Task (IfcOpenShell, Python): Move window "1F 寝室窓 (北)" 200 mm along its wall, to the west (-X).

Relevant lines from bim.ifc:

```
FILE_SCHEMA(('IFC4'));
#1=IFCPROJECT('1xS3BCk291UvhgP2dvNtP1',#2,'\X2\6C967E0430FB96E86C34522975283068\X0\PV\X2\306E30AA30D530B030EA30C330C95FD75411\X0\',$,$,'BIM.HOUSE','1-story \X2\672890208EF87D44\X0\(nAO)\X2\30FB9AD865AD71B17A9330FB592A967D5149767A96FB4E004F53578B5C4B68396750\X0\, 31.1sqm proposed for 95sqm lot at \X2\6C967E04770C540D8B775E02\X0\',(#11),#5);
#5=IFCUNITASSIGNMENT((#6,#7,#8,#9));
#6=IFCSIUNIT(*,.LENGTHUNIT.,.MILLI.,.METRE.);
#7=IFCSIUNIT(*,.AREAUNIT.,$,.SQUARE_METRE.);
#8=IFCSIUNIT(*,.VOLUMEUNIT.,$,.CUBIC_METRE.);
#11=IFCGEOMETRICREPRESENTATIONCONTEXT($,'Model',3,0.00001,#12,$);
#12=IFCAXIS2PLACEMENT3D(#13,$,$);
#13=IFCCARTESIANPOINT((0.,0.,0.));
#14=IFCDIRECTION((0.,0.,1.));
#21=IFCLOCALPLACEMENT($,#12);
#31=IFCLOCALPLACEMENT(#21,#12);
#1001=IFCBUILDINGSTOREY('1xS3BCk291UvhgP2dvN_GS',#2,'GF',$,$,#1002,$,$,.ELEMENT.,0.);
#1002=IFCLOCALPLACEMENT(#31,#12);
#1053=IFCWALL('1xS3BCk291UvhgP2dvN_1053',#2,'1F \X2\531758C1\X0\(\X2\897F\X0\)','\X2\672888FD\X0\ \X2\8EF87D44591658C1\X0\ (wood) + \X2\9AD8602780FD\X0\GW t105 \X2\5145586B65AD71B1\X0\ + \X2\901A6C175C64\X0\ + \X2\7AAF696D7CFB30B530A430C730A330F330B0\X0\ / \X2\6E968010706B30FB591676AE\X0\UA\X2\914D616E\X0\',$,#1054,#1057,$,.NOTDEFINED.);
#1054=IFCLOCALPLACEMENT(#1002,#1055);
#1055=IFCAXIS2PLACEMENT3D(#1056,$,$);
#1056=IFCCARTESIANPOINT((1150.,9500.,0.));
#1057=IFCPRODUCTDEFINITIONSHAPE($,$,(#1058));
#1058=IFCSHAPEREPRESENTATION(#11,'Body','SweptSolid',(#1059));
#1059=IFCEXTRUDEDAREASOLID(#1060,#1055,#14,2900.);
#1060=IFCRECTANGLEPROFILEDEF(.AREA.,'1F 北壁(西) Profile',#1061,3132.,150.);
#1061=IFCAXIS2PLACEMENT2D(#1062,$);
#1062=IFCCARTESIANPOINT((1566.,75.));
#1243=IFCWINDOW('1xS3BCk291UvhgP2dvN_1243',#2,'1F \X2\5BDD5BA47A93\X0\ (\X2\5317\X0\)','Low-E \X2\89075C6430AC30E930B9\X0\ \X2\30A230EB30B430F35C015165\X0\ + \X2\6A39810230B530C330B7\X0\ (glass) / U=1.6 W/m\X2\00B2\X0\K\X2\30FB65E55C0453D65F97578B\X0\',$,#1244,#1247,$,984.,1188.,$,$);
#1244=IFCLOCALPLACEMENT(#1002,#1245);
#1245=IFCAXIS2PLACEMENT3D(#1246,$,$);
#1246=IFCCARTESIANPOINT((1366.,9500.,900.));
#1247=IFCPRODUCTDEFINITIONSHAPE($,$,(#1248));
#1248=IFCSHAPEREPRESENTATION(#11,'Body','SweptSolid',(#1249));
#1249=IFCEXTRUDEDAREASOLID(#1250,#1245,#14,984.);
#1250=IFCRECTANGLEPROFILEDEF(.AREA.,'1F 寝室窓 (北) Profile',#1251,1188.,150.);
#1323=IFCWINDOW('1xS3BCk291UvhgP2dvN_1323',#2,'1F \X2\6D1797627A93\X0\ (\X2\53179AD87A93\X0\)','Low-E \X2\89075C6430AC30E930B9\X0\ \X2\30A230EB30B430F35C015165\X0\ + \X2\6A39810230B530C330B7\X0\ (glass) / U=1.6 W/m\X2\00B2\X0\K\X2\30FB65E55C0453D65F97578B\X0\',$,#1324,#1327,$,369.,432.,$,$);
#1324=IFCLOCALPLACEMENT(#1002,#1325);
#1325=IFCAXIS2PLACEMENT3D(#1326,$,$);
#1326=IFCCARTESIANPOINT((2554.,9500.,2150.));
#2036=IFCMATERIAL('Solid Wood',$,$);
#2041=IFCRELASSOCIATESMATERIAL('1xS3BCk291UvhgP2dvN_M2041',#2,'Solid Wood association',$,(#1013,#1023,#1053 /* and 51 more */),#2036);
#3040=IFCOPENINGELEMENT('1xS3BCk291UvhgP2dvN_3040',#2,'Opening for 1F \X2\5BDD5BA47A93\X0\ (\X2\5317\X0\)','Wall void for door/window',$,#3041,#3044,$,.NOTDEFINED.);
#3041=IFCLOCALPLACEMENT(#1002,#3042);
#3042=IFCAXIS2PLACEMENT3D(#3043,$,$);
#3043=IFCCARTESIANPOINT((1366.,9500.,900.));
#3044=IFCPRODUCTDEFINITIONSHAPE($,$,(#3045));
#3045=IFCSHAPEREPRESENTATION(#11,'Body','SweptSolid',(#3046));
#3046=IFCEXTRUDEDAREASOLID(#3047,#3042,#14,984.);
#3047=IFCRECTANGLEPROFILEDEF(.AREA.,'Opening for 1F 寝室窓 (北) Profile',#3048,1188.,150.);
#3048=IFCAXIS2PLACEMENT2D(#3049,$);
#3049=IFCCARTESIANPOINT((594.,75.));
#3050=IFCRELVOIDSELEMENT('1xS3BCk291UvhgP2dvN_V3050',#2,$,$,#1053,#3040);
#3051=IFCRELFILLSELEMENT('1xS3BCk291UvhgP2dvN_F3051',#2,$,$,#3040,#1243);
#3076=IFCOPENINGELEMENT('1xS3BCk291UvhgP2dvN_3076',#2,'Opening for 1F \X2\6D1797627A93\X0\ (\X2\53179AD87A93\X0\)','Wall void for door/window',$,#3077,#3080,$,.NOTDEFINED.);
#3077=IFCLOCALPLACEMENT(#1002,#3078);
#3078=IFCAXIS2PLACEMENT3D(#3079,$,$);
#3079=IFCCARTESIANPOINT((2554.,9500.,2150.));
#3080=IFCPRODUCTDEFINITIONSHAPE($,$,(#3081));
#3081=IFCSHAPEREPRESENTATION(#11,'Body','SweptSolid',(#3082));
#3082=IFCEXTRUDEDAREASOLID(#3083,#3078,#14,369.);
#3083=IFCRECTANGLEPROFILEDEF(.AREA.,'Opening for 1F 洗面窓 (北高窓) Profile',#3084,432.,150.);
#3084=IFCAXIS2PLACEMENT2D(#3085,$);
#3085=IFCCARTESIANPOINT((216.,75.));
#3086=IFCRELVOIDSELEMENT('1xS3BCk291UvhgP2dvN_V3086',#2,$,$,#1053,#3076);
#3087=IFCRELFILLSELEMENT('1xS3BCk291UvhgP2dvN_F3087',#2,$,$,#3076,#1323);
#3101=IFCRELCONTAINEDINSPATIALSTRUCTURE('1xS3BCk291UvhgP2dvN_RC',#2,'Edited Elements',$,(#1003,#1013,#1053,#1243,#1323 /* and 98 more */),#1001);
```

```python
import ifcopenshell
import ifcopenshell.api.geometry
import ifcopenshell.util.placement
import ifcopenshell.util.unit

model = ifcopenshell.open("bim.ifc")
unit_scale = ifcopenshell.util.unit.calculate_unit_scale(model)

window = model.by_guid("1xS3BCk291UvhgP2dvN_1243")
opening = window.FillsVoids[0].RelatingOpeningElement
wall = opening.VoidsElements[0].RelatingBuildingElement

wall_matrix = ifcopenshell.util.placement.get_local_placement(wall.ObjectPlacement)
shift = wall_matrix[:3, 0] * -0.2 / unit_scale
before = ifcopenshell.util.placement.get_local_placement(window.ObjectPlacement)[:3, 3].copy()

# The window is not placed relative to its opening, so move both.
for product in (opening, window):
    matrix = ifcopenshell.util.placement.get_local_placement(product.ObjectPlacement)
    matrix[:3, 3] += shift
    ifcopenshell.api.geometry.edit_object_placement(model, product=product, matrix=matrix, is_si=False)

after = ifcopenshell.util.placement.get_local_placement(window.ObjectPlacement)[:3, 3]
print("window moved by", (after - before).round(3) + 0.0)

model.write("bim-out.ifc")
```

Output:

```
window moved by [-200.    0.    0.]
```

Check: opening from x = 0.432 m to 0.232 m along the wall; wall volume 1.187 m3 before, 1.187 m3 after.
